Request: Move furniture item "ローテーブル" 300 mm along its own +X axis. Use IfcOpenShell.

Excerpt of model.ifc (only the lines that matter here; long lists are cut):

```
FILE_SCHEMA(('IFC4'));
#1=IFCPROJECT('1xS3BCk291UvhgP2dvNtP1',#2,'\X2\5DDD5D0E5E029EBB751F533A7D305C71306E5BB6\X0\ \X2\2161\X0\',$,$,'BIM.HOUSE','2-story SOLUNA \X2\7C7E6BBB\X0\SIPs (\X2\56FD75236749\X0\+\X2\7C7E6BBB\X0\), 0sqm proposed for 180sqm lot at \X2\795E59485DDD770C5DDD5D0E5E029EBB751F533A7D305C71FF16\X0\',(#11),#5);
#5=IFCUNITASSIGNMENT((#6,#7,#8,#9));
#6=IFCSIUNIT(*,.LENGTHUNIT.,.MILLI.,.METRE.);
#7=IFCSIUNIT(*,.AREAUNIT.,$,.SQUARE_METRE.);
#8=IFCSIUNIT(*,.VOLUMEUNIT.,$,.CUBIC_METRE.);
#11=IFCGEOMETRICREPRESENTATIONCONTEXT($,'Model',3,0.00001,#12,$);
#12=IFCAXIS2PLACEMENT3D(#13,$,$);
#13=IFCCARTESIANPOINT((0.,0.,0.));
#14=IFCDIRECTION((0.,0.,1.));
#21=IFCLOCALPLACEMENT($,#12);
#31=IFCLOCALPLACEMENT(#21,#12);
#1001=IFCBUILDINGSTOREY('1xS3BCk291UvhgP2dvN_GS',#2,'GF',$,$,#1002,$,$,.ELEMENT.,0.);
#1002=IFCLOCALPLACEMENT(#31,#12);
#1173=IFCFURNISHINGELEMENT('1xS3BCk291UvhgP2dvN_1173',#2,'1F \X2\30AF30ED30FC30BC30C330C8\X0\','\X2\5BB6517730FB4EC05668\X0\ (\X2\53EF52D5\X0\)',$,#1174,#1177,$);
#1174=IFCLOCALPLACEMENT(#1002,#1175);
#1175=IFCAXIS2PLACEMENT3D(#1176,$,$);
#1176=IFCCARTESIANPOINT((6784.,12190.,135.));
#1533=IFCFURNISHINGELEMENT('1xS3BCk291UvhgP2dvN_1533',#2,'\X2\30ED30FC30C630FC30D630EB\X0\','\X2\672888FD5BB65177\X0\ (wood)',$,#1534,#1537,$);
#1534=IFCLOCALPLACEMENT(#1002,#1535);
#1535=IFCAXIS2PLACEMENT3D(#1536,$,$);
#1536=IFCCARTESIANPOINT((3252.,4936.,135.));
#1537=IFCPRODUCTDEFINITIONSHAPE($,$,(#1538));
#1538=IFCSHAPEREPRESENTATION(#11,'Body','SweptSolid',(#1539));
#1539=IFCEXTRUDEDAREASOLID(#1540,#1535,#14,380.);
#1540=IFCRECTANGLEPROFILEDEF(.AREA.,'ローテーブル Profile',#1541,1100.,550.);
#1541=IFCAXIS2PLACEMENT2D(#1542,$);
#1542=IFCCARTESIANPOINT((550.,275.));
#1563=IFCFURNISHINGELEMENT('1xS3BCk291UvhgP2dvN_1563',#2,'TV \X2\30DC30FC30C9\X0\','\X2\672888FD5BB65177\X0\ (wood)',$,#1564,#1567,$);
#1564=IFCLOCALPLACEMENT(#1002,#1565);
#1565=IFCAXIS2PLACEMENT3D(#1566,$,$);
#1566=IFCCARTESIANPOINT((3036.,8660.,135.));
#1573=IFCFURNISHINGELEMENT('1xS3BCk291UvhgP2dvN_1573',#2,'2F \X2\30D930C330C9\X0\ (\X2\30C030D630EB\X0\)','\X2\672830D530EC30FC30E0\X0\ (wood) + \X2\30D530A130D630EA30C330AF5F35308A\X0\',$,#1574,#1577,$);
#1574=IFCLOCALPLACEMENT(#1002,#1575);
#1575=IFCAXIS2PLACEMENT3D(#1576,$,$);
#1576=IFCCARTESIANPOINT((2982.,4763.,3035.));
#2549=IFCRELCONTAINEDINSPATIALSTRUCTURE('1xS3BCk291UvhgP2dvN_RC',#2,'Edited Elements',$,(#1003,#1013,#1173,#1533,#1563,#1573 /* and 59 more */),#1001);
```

```python
import ifcopenshell
import ifcopenshell.api.geometry
import ifcopenshell.util.placement
import ifcopenshell.util.unit

model = ifcopenshell.open("model.ifc")
unit_scale = ifcopenshell.util.unit.calculate_unit_scale(model)

item = model.by_id(1533)
matrix = ifcopenshell.util.placement.get_local_placement(item.ObjectPlacement)
matrix[:3, 3] += matrix[:3, 0] * 0.3 / unit_scale
ifcopenshell.api.geometry.edit_object_placement(model, product=item, matrix=matrix, is_si=False)

print(ifcopenshell.util.placement.get_local_placement(item.ObjectPlacement).round(3) + 0.0)

model.write("model_updated.ifc")
```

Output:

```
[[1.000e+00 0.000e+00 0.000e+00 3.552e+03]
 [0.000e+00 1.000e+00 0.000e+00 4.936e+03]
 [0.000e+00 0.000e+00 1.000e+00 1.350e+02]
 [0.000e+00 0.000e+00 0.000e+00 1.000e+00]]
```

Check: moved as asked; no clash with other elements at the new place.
